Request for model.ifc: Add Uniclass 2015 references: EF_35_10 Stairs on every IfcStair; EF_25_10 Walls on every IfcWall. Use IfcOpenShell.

First a look at what the model holds.

```python
import ifcopenshell

model = ifcopenshell.open("model.ifc")
print(model.schema)
print("classifications:", [c.Name for c in model.by_type("IfcClassification")])
for ifc_class in ("IfcDoor", "IfcRoof", "IfcStair", "IfcWall", "IfcWindow"):
    print(ifc_class, len(model.by_type(ifc_class)))
```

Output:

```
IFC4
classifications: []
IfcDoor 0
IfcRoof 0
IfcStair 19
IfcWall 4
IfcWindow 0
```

```python
import ifcopenshell
import ifcopenshell.api.classification

model = ifcopenshell.open("model.ifc")

system = ifcopenshell.api.classification.add_classification(model, classification="Uniclass 2015")

codes = {
    "IfcStair": ("EF_35_10", "Stairs"),
    "IfcWall": ("EF_25_10", "Walls"),
}
for ifc_class, (code, name) in codes.items():
    products = model.by_type(ifc_class)
    ifcopenshell.api.classification.add_reference(
        model, products=products, classification=system, identification=code, name=name
    )
    print(code, len(products))

model.write("model_updated.ifc")
```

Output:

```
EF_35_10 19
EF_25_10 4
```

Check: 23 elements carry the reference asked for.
